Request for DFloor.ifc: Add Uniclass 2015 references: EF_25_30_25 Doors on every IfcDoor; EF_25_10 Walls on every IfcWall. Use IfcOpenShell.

First a look at what the model holds.

```python
import ifcopenshell

model = ifcopenshell.open("DFloor.ifc")
print(model.schema)
print("classifications:", [c.Name for c in model.by_type("IfcClassification")])
for ifc_class in ("IfcDoor", "IfcRoof", "IfcStair", "IfcWall", "IfcWindow"):
    print(ifc_class, len(model.by_type(ifc_class)))
```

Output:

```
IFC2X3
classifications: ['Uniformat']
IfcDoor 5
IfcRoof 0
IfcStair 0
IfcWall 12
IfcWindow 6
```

```python
import ifcopenshell
import ifcopenshell.api.classification

model = ifcopenshell.open("DFloor.ifc")

# IFC2X3 requires Source and Edition and has no link from the project to the system.
system = model.create_entity("IfcClassification", Source="NBS", Edition="2015", Name="Uniclass 2015")

codes = {
    "IfcDoor": ("EF_25_30_25", "Doors"),
    "IfcWall": ("EF_25_10", "Walls"),
}
for ifc_class, (code, name) in codes.items():
    products = model.by_type(ifc_class)
    ifcopenshell.api.classification.add_reference(
        model, products=products, classification=system, identification=code, name=name
    )
    print(code, len(products))

model.write("DFloor-out.ifc")
```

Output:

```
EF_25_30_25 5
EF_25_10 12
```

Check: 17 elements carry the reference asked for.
